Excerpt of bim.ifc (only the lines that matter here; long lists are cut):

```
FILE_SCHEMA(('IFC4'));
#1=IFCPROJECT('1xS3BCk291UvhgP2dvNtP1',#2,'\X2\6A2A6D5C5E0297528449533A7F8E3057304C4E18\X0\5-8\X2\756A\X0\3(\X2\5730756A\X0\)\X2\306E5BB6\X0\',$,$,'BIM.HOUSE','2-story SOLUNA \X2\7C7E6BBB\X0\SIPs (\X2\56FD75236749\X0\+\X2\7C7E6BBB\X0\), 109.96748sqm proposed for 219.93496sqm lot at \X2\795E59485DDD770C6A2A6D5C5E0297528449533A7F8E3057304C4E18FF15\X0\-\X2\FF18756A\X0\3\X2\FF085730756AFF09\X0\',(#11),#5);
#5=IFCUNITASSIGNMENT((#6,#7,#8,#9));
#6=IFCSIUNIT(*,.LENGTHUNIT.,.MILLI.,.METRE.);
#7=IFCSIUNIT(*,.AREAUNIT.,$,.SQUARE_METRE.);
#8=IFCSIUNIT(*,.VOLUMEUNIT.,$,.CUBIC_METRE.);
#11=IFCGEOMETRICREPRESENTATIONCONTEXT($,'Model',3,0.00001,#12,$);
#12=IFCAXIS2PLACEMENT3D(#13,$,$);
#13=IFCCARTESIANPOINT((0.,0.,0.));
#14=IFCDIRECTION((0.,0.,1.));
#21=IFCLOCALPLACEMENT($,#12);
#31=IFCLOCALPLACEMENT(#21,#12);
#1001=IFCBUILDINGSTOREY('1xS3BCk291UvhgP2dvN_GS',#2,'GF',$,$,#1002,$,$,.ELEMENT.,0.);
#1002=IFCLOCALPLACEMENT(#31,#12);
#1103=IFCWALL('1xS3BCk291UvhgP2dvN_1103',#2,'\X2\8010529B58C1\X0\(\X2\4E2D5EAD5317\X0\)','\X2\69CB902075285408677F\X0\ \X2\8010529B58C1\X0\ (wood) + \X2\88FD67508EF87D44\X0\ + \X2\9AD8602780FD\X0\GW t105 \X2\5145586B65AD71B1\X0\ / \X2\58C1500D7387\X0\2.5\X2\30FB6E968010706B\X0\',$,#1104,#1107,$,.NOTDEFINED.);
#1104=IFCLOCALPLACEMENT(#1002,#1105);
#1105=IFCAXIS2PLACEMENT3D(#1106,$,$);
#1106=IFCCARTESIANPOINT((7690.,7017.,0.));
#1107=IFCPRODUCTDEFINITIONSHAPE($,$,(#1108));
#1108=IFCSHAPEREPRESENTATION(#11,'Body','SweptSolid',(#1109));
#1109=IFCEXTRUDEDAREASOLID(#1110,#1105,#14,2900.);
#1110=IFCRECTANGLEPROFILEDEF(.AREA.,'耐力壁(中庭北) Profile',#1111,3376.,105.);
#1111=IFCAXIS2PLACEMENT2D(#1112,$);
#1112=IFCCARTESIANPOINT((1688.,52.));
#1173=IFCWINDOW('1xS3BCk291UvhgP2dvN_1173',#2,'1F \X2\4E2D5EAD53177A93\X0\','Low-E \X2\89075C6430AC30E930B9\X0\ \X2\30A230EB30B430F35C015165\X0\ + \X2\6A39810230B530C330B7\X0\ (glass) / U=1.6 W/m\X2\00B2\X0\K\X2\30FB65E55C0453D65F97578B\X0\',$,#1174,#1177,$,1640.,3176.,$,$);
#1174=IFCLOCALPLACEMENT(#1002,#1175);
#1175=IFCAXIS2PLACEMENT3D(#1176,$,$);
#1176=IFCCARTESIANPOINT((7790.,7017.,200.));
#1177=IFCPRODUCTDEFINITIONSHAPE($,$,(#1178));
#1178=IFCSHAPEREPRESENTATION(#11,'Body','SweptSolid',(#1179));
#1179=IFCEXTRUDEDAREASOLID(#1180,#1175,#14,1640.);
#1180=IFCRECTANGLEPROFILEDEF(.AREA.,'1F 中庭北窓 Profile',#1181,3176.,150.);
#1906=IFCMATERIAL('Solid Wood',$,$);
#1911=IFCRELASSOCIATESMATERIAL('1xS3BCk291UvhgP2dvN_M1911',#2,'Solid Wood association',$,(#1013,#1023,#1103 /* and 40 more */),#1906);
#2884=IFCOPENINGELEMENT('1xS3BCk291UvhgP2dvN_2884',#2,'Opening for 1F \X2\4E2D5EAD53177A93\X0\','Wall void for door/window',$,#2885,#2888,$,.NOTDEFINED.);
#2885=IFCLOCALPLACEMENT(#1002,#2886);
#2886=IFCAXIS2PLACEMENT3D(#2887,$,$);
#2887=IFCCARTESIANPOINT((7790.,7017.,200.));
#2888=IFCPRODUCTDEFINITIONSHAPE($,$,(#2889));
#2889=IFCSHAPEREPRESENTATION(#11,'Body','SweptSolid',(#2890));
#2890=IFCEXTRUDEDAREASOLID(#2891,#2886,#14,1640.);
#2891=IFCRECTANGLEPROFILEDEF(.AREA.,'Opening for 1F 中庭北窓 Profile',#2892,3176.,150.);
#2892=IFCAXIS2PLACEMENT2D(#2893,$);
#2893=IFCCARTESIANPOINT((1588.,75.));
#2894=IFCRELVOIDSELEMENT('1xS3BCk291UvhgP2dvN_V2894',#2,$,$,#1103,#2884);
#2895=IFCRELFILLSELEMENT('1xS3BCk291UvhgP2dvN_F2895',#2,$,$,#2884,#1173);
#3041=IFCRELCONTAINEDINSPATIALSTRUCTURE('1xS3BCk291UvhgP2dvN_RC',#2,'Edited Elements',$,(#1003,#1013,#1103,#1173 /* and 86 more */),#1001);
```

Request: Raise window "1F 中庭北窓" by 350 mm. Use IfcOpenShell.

```python
import numpy as np
import ifcopenshell
import ifcopenshell.api.geometry
import ifcopenshell.util.placement
import ifcopenshell.util.unit

model = ifcopenshell.open("bim.ifc")
unit_scale = ifcopenshell.util.unit.calculate_unit_scale(model)

window = model.by_guid("1xS3BCk291UvhgP2dvN_1173")
opening = window.FillsVoids[0].RelatingOpeningElement
dz = 0.35 / unit_scale

shift = np.array([0.0, 0.0, dz])
# The window is not placed relative to its opening, so move both.
for product in (opening, window):
    matrix = ifcopenshell.util.placement.get_local_placement(product.ObjectPlacement)
    matrix[:3, 3] += shift
    ifcopenshell.api.geometry.edit_object_placement(model, product=product, matrix=matrix, is_si=False)

print(f"moved by {dz * unit_scale:+.3f} m")

model.write("bim_rev.ifc")
```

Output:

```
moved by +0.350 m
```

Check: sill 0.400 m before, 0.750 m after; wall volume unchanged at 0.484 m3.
